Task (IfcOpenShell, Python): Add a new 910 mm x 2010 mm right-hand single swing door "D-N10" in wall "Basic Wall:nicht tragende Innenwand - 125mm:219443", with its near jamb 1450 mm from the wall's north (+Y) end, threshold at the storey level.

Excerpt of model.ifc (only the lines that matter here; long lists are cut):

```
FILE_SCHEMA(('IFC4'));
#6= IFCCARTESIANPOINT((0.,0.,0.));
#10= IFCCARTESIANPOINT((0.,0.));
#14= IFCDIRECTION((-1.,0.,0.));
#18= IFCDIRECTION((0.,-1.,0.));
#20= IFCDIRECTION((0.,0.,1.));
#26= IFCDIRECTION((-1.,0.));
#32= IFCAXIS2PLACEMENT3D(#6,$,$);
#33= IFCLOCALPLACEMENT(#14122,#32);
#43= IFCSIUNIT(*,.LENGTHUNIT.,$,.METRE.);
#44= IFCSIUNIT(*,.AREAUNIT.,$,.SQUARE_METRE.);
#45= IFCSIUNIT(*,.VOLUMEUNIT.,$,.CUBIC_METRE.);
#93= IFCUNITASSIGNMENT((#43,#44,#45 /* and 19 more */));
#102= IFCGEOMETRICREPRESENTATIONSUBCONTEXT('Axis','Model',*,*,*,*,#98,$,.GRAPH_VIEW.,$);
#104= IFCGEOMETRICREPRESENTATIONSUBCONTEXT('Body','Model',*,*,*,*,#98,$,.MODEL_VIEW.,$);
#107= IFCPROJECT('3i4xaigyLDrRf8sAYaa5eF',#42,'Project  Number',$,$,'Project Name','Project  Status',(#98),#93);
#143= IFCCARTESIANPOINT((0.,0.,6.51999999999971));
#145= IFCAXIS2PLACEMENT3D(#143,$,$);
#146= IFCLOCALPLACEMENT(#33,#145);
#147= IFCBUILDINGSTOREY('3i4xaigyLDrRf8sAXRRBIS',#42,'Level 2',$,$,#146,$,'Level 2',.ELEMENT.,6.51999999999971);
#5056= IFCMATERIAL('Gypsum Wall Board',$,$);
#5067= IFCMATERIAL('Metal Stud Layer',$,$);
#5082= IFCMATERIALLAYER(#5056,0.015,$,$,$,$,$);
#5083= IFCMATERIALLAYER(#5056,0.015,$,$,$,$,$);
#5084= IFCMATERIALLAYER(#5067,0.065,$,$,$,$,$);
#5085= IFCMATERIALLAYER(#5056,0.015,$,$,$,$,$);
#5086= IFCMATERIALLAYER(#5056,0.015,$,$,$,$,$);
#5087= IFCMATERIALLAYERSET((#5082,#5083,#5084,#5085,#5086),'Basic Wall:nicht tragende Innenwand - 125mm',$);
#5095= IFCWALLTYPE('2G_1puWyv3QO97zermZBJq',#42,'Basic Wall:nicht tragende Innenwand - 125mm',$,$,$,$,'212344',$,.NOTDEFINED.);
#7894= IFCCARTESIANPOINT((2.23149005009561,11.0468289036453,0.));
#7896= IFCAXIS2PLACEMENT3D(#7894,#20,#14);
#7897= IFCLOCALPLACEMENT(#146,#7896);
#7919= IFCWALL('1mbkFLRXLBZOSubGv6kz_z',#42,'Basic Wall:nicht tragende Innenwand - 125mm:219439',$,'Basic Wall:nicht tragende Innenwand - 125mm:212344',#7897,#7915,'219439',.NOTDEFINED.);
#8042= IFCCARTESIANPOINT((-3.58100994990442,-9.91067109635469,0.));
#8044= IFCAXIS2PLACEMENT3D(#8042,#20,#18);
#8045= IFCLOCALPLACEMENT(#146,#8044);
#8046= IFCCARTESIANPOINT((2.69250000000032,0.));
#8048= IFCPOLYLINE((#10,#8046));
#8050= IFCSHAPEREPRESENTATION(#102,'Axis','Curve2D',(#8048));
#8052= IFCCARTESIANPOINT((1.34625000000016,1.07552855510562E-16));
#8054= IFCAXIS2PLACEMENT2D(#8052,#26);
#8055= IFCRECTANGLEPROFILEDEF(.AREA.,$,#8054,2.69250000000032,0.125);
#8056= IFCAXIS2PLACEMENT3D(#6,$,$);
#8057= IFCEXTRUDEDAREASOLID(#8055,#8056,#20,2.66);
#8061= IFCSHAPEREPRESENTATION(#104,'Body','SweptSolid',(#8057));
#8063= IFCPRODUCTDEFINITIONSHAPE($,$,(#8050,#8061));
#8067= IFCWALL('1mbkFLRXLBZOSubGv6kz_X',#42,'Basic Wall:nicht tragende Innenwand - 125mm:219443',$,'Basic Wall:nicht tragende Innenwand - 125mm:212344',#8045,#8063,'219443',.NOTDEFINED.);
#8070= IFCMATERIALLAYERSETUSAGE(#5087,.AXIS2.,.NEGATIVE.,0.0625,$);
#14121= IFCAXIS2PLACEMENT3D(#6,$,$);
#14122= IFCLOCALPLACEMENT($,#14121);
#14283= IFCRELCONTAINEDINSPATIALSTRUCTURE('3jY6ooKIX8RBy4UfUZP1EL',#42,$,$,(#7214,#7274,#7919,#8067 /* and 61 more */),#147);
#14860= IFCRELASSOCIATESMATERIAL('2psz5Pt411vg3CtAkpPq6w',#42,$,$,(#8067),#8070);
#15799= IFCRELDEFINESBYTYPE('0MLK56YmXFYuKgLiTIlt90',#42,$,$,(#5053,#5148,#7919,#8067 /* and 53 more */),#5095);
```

```python
import numpy as np
import ifcopenshell
import ifcopenshell.api.feature
import ifcopenshell.api.geometry
import ifcopenshell.api.root
import ifcopenshell.api.spatial
import ifcopenshell.geom
import ifcopenshell.util.element
import ifcopenshell.util.placement
import ifcopenshell.util.representation
import ifcopenshell.util.shape
import ifcopenshell.util.unit

model = ifcopenshell.open("model.ifc")
unit_scale = ifcopenshell.util.unit.calculate_unit_scale(model)
settings = ifcopenshell.geom.settings()


def volume(element):
    """Net volume in cubic metres, openings subtracted."""
    shape = ifcopenshell.geom.create_shape(settings, element)
    return ifcopenshell.util.shape.get_volume(shape.geometry)


wall = model.by_id(8067)
storey = ifcopenshell.util.element.get_container(wall, ifc_class="IfcBuildingStorey")
context = ifcopenshell.util.representation.get_context(model, "Model", "Body", "MODEL_VIEW")
before = volume(wall)

width, height, from_end, sill = 0.91, 2.01, 1.45, 0.0  # metres

# The wall runs along its own X axis, and the end named is its -X end.
wall_shape = ifcopenshell.geom.create_shape(settings, wall)
x, y, z = ifcopenshell.util.shape.get_vertices(wall_shape.geometry).T
start = x.min() + from_end
face, thickness = float(y.min()), float(y.max() - y.min())
wall_matrix = ifcopenshell.util.placement.get_local_placement(wall.ObjectPlacement)
level = ifcopenshell.util.placement.get_local_placement(storey.ObjectPlacement)[2, 3]


def in_wall(x, y):
    """Placement at x, y metres in the wall's axes, at sill height."""
    matrix = wall_matrix.copy()
    matrix[:, 3] = wall_matrix @ np.array([x / unit_scale, y / unit_scale, 0.0, 1.0])
    matrix[2, 3] = level + sill / unit_scale
    return matrix


# Opening: a box that overshoots both wall faces by 50 mm.
opening = ifcopenshell.api.root.create_entity(model, ifc_class="IfcOpeningElement", predefined_type="OPENING")
box = ifcopenshell.api.geometry.add_wall_representation(
    model, context=context, length=width, height=height, thickness=thickness + 0.1
)
ifcopenshell.api.geometry.assign_representation(model, product=opening, representation=box)
ifcopenshell.api.geometry.edit_object_placement(model, product=opening, matrix=in_wall(start, face - 0.05), is_si=False)
ifcopenshell.api.feature.add_feature(model, feature=opening, element=wall)

door = ifcopenshell.api.root.create_entity(model, ifc_class="IfcDoor", name="D-N10", predefined_type="DOOR")
door.OverallWidth, door.OverallHeight = width / unit_scale, height / unit_scale
door.OperationType = "SINGLE_SWING_RIGHT"
body = ifcopenshell.api.geometry.add_door_representation(
    model,
    context=context,
    overall_width=door.OverallWidth,
    overall_height=door.OverallHeight,
    operation_type="SINGLE_SWING_RIGHT",
    lining_properties={"LiningDepth": thickness / unit_scale, "ThresholdDepth": thickness / unit_scale},
)
ifcopenshell.api.geometry.assign_representation(model, product=door, representation=body)
ifcopenshell.api.spatial.assign_container(model, products=[door], relating_structure=storey)
ifcopenshell.api.feature.add_filling(model, opening=opening, element=door)

# The lining spans the wall, so the door starts at the wall face.
ifcopenshell.api.geometry.edit_object_placement(model, product=door, matrix=in_wall(start, face), is_si=False)

after = volume(wall)

print(f"wall volume {before:.3f} -> {after:.3f} m3")

model.write("model_updated.ifc")
```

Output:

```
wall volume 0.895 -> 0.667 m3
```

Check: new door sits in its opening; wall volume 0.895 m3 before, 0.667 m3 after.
